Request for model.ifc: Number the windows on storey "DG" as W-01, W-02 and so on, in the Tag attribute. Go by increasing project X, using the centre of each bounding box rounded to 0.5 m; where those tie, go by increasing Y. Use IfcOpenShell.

First a look at what the model holds.

```python
import ifcopenshell
import ifcopenshell.util.element
import ifcopenshell.util.placement

model = ifcopenshell.open("model.ifc")
print(model.schema)
storey = next(s for s in model.by_type("IfcBuildingStorey") if s.Name == "DG")
windows = [e for e in ifcopenshell.util.element.get_decomposition(storey) if e.is_a("IfcWindow")]
for e in sorted(windows, key=lambda e: e.id()):
    origin = ifcopenshell.util.placement.get_local_placement(e.ObjectPlacement)[:3, 3]
    print(e.id(), e.Tag, e.Name, origin.round(2) + 0.0, sep=" | ")
```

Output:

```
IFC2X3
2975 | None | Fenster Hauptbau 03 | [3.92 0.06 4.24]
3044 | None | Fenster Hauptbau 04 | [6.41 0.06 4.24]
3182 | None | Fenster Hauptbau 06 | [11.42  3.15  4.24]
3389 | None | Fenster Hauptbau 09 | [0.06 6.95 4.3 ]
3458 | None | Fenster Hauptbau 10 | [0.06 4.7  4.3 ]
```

```python
import ifcopenshell
import ifcopenshell.geom
import ifcopenshell.util.element
import ifcopenshell.util.shape

model = ifcopenshell.open("model.ifc")
settings = ifcopenshell.geom.settings()
settings.set("use-world-coords", True)


def centre(element):
    shape = ifcopenshell.geom.create_shape(settings, element)
    return ifcopenshell.util.shape.get_bbox_centroid(shape.geometry)


storey = next(s for s in model.by_type("IfcBuildingStorey") if s.Name == "DG")
windows = [e for e in ifcopenshell.util.element.get_decomposition(storey) if e.is_a("IfcWindow")]

# Insertion points can sit at a corner or the storey origin, so sort by the geometry (in metres).
centres = {e: centre(e) for e in windows}
windows.sort(key=lambda e: (round(centres[e][0] / 0.5), centres[e][1]))

for i, e in enumerate(windows, start=1):
    number = f"W-{i:02d}"
    e.Tag = number
    print(e.id(), number)

model.write("model_rev.ifc")
```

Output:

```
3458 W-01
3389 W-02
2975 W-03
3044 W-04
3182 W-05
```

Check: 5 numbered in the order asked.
